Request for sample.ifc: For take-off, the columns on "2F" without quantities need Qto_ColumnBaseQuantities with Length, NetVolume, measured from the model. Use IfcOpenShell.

First a look at what the model holds.

```python
import ifcopenshell
import ifcopenshell.util.element
import ifcopenshell.util.unit

model = ifcopenshell.open("sample.ifc")
print(model.schema)
for unit_type in ("LENGTHUNIT", "AREAUNIT", "VOLUMEUNIT"):
    print(unit_type, ifcopenshell.util.unit.calculate_unit_scale(model, unit_type))
storey = next(s for s in model.by_type("IfcBuildingStorey") if s.Name == "2F")
columns = [e for e in ifcopenshell.util.element.get_decomposition(storey) if e.is_a("IfcColumn")]
for e in sorted(columns, key=lambda e: e.id()):
    print(e.id(), e.is_a(), e.Name, list(ifcopenshell.util.element.get_psets(e, qtos_only=True)), sep=" | ")
```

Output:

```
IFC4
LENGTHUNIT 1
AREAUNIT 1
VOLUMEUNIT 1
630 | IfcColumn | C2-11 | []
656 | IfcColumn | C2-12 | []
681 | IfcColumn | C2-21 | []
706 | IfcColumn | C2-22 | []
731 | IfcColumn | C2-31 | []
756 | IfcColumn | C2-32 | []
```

```python
import ifcopenshell
import ifcopenshell.api.pset
import ifcopenshell.geom
import ifcopenshell.util.element
import ifcopenshell.util.shape
import ifcopenshell.util.unit

model = ifcopenshell.open("sample.ifc")
unit_scale = ifcopenshell.util.unit.calculate_unit_scale(model)
volume_scale = ifcopenshell.util.unit.calculate_unit_scale(model, "VOLUMEUNIT")
settings = ifcopenshell.geom.settings()

storey = next(s for s in model.by_type("IfcBuildingStorey") if s.Name == "2F")
columns = [e for e in ifcopenshell.util.element.get_decomposition(storey) if e.is_a("IfcColumn")]

for e in sorted(columns, key=lambda e: e.id()):
    if ifcopenshell.util.element.get_psets(e, qtos_only=True, should_inherit=False):
        continue
    # Geometry comes back in metres, in the element's own axes.
    shape = ifcopenshell.geom.create_shape(settings, e)
    values = {
        "Length": ifcopenshell.util.shape.get_z(shape.geometry) / unit_scale,
        "NetVolume": ifcopenshell.util.shape.get_volume(shape.geometry) / volume_scale,
    }
    qto = ifcopenshell.api.pset.add_qto(model, product=e, name="Qto_ColumnBaseQuantities")
    ifcopenshell.api.pset.edit_qto(model, qto=qto, properties=values)
    print(e.id(), {k: round(v, 3) for k, v in values.items()})

model.write("sample-out.ifc")
```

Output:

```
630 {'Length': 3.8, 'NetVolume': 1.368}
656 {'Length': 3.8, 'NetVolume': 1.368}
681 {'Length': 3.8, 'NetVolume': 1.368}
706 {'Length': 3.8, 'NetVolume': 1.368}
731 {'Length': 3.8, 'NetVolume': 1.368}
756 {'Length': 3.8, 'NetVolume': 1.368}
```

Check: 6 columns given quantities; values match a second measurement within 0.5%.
